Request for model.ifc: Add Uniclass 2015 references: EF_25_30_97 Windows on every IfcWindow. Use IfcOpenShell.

First a look at what the model holds.

```python
import ifcopenshell

model = ifcopenshell.open("model.ifc")
print(model.schema)
print("classifications:", [c.Name for c in model.by_type("IfcClassification")])
for ifc_class in ("IfcDoor", "IfcRoof", "IfcStair", "IfcWall", "IfcWindow"):
    print(ifc_class, len(model.by_type(ifc_class)))
```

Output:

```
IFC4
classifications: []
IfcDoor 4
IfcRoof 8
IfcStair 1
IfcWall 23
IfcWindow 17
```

```python
import ifcopenshell
import ifcopenshell.api.classification

model = ifcopenshell.open("model.ifc")

system = ifcopenshell.api.classification.add_classification(model, classification="Uniclass 2015")

codes = {
    "IfcWindow": ("EF_25_30_97", "Windows"),
}
for ifc_class, (code, name) in codes.items():
    products = model.by_type(ifc_class)
    ifcopenshell.api.classification.add_reference(
        model, products=products, classification=system, identification=code, name=name
    )
    print(code, len(products))

model.write("model_rev.ifc")
```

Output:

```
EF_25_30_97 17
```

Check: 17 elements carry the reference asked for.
